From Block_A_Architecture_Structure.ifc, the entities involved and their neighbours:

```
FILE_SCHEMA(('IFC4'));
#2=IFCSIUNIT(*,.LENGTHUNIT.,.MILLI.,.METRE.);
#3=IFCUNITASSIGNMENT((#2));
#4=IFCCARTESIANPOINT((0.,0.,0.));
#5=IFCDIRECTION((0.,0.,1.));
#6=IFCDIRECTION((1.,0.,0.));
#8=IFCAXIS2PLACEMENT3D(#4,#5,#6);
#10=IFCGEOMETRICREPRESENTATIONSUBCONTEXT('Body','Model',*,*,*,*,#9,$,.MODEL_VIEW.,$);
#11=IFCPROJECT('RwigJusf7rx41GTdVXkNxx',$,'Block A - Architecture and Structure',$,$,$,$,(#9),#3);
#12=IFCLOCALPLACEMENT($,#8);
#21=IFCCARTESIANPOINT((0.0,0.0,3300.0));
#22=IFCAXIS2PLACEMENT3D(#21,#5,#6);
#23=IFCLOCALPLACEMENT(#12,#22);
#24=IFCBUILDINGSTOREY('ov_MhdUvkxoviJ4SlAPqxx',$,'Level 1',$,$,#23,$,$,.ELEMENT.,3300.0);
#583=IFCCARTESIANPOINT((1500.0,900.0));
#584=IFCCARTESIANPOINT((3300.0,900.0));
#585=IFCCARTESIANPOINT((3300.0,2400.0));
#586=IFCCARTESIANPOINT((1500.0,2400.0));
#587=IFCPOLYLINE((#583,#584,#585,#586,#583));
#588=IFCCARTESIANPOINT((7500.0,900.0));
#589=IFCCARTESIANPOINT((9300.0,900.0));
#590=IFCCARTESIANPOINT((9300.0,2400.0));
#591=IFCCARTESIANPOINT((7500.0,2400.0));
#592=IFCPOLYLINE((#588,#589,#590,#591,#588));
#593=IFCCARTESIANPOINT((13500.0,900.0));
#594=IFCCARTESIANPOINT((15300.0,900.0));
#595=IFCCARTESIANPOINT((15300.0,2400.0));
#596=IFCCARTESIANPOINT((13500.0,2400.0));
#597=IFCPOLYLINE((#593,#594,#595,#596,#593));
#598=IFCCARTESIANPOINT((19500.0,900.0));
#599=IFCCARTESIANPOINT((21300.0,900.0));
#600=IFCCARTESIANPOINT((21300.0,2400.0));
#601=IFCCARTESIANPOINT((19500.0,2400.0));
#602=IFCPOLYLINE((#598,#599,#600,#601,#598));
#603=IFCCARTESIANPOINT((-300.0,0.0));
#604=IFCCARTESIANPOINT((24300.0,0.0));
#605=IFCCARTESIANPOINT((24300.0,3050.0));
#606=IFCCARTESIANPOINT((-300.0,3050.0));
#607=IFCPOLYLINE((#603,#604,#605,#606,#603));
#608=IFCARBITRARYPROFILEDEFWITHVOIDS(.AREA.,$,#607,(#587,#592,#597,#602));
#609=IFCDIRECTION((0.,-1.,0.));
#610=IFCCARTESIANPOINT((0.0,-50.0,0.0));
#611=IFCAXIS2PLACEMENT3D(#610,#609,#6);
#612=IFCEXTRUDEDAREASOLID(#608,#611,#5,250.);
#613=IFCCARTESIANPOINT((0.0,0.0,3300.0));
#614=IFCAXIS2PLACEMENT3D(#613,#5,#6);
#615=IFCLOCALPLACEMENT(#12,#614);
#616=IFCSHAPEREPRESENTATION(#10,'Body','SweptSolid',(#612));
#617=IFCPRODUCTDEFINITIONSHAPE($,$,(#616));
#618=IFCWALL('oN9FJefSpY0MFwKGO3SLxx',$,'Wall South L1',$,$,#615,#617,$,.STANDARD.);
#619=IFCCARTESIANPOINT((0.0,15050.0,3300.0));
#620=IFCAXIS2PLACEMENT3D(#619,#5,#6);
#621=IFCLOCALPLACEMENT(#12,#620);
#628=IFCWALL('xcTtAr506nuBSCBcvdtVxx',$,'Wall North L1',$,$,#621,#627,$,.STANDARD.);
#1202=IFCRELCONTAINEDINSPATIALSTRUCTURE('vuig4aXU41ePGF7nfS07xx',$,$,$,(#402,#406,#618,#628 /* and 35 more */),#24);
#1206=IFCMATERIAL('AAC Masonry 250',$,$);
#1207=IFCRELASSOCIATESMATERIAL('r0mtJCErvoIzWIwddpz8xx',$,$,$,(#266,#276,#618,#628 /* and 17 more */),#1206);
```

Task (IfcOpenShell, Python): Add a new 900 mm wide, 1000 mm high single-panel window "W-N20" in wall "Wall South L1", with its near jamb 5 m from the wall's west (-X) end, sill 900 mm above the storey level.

```python
import numpy as np
import ifcopenshell
import ifcopenshell.api.feature
import ifcopenshell.api.geometry
import ifcopenshell.api.root
import ifcopenshell.api.spatial
import ifcopenshell.geom
import ifcopenshell.util.element
import ifcopenshell.util.placement
import ifcopenshell.util.representation
import ifcopenshell.util.shape
import ifcopenshell.util.unit

model = ifcopenshell.open("Block_A_Architecture_Structure.ifc")
unit_scale = ifcopenshell.util.unit.calculate_unit_scale(model)
settings = ifcopenshell.geom.settings()


def volume(element):
    """Net volume in cubic metres, openings subtracted."""
    shape = ifcopenshell.geom.create_shape(settings, element)
    return ifcopenshell.util.shape.get_volume(shape.geometry)


wall = model.by_id(618)
storey = ifcopenshell.util.element.get_container(wall, ifc_class="IfcBuildingStorey")
context = ifcopenshell.util.representation.get_context(model, "Model", "Body", "MODEL_VIEW")
before = volume(wall)

width, height, from_end, sill = 0.9, 1, 5, 0.9  # metres

# The wall runs along its own X axis, and the end named is its -X end.
wall_shape = ifcopenshell.geom.create_shape(settings, wall)
x, y, z = ifcopenshell.util.shape.get_vertices(wall_shape.geometry).T
start = x.min() + from_end
face, thickness = float(y.min()), float(y.max() - y.min())
wall_matrix = ifcopenshell.util.placement.get_local_placement(wall.ObjectPlacement)
level = ifcopenshell.util.placement.get_local_placement(storey.ObjectPlacement)[2, 3]


def in_wall(x, y):
    """Placement at x, y metres in the wall's axes, at sill height."""
    matrix = wall_matrix.copy()
    matrix[:, 3] = wall_matrix @ np.array([x / unit_scale, y / unit_scale, 0.0, 1.0])
    matrix[2, 3] = level + sill / unit_scale
    return matrix


# Opening: a box that overshoots both wall faces by 50 mm.
opening = ifcopenshell.api.root.create_entity(model, ifc_class="IfcOpeningElement", predefined_type="OPENING")
box = ifcopenshell.api.geometry.add_wall_representation(
    model, context=context, length=width, height=height, thickness=thickness + 0.1
)
ifcopenshell.api.geometry.assign_representation(model, product=opening, representation=box)
ifcopenshell.api.geometry.edit_object_placement(model, product=opening, matrix=in_wall(start, face - 0.05), is_si=False)
ifcopenshell.api.feature.add_feature(model, feature=opening, element=wall)

window = ifcopenshell.api.root.create_entity(model, ifc_class="IfcWindow", name="W-N20", predefined_type="WINDOW")
window.OverallWidth, window.OverallHeight = width / unit_scale, height / unit_scale
window.PartitioningType = "SINGLE_PANEL"
body = ifcopenshell.api.geometry.add_window_representation(
    model,
    context=context,
    overall_width=window.OverallWidth,
    overall_height=window.OverallHeight,
    partition_type="SINGLE_PANEL",
)
ifcopenshell.api.geometry.assign_representation(model, product=window, representation=body)
ifcopenshell.api.spatial.assign_container(model, products=[window], relating_structure=storey)
ifcopenshell.api.feature.add_filling(model, opening=opening, element=window)

# Centre the window in the wall's thickness.
ifcopenshell.api.geometry.edit_object_placement(model, product=window, matrix=in_wall(start, face), is_si=False)
window_shape = ifcopenshell.geom.create_shape(settings, window)
depth = ifcopenshell.util.shape.get_vertices(window_shape.geometry)[:, 1]
offset = face + thickness / 2 - (depth.min() + depth.max()) / 2
ifcopenshell.api.geometry.edit_object_placement(model, product=window, matrix=in_wall(start, offset), is_si=False)

after = volume(wall)

print(f"wall volume {before:.3f} -> {after:.3f} m3")

model.write("Block_A_Architecture_Structure_rev.ifc")
```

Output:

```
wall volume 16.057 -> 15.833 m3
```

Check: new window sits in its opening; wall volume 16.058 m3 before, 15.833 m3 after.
